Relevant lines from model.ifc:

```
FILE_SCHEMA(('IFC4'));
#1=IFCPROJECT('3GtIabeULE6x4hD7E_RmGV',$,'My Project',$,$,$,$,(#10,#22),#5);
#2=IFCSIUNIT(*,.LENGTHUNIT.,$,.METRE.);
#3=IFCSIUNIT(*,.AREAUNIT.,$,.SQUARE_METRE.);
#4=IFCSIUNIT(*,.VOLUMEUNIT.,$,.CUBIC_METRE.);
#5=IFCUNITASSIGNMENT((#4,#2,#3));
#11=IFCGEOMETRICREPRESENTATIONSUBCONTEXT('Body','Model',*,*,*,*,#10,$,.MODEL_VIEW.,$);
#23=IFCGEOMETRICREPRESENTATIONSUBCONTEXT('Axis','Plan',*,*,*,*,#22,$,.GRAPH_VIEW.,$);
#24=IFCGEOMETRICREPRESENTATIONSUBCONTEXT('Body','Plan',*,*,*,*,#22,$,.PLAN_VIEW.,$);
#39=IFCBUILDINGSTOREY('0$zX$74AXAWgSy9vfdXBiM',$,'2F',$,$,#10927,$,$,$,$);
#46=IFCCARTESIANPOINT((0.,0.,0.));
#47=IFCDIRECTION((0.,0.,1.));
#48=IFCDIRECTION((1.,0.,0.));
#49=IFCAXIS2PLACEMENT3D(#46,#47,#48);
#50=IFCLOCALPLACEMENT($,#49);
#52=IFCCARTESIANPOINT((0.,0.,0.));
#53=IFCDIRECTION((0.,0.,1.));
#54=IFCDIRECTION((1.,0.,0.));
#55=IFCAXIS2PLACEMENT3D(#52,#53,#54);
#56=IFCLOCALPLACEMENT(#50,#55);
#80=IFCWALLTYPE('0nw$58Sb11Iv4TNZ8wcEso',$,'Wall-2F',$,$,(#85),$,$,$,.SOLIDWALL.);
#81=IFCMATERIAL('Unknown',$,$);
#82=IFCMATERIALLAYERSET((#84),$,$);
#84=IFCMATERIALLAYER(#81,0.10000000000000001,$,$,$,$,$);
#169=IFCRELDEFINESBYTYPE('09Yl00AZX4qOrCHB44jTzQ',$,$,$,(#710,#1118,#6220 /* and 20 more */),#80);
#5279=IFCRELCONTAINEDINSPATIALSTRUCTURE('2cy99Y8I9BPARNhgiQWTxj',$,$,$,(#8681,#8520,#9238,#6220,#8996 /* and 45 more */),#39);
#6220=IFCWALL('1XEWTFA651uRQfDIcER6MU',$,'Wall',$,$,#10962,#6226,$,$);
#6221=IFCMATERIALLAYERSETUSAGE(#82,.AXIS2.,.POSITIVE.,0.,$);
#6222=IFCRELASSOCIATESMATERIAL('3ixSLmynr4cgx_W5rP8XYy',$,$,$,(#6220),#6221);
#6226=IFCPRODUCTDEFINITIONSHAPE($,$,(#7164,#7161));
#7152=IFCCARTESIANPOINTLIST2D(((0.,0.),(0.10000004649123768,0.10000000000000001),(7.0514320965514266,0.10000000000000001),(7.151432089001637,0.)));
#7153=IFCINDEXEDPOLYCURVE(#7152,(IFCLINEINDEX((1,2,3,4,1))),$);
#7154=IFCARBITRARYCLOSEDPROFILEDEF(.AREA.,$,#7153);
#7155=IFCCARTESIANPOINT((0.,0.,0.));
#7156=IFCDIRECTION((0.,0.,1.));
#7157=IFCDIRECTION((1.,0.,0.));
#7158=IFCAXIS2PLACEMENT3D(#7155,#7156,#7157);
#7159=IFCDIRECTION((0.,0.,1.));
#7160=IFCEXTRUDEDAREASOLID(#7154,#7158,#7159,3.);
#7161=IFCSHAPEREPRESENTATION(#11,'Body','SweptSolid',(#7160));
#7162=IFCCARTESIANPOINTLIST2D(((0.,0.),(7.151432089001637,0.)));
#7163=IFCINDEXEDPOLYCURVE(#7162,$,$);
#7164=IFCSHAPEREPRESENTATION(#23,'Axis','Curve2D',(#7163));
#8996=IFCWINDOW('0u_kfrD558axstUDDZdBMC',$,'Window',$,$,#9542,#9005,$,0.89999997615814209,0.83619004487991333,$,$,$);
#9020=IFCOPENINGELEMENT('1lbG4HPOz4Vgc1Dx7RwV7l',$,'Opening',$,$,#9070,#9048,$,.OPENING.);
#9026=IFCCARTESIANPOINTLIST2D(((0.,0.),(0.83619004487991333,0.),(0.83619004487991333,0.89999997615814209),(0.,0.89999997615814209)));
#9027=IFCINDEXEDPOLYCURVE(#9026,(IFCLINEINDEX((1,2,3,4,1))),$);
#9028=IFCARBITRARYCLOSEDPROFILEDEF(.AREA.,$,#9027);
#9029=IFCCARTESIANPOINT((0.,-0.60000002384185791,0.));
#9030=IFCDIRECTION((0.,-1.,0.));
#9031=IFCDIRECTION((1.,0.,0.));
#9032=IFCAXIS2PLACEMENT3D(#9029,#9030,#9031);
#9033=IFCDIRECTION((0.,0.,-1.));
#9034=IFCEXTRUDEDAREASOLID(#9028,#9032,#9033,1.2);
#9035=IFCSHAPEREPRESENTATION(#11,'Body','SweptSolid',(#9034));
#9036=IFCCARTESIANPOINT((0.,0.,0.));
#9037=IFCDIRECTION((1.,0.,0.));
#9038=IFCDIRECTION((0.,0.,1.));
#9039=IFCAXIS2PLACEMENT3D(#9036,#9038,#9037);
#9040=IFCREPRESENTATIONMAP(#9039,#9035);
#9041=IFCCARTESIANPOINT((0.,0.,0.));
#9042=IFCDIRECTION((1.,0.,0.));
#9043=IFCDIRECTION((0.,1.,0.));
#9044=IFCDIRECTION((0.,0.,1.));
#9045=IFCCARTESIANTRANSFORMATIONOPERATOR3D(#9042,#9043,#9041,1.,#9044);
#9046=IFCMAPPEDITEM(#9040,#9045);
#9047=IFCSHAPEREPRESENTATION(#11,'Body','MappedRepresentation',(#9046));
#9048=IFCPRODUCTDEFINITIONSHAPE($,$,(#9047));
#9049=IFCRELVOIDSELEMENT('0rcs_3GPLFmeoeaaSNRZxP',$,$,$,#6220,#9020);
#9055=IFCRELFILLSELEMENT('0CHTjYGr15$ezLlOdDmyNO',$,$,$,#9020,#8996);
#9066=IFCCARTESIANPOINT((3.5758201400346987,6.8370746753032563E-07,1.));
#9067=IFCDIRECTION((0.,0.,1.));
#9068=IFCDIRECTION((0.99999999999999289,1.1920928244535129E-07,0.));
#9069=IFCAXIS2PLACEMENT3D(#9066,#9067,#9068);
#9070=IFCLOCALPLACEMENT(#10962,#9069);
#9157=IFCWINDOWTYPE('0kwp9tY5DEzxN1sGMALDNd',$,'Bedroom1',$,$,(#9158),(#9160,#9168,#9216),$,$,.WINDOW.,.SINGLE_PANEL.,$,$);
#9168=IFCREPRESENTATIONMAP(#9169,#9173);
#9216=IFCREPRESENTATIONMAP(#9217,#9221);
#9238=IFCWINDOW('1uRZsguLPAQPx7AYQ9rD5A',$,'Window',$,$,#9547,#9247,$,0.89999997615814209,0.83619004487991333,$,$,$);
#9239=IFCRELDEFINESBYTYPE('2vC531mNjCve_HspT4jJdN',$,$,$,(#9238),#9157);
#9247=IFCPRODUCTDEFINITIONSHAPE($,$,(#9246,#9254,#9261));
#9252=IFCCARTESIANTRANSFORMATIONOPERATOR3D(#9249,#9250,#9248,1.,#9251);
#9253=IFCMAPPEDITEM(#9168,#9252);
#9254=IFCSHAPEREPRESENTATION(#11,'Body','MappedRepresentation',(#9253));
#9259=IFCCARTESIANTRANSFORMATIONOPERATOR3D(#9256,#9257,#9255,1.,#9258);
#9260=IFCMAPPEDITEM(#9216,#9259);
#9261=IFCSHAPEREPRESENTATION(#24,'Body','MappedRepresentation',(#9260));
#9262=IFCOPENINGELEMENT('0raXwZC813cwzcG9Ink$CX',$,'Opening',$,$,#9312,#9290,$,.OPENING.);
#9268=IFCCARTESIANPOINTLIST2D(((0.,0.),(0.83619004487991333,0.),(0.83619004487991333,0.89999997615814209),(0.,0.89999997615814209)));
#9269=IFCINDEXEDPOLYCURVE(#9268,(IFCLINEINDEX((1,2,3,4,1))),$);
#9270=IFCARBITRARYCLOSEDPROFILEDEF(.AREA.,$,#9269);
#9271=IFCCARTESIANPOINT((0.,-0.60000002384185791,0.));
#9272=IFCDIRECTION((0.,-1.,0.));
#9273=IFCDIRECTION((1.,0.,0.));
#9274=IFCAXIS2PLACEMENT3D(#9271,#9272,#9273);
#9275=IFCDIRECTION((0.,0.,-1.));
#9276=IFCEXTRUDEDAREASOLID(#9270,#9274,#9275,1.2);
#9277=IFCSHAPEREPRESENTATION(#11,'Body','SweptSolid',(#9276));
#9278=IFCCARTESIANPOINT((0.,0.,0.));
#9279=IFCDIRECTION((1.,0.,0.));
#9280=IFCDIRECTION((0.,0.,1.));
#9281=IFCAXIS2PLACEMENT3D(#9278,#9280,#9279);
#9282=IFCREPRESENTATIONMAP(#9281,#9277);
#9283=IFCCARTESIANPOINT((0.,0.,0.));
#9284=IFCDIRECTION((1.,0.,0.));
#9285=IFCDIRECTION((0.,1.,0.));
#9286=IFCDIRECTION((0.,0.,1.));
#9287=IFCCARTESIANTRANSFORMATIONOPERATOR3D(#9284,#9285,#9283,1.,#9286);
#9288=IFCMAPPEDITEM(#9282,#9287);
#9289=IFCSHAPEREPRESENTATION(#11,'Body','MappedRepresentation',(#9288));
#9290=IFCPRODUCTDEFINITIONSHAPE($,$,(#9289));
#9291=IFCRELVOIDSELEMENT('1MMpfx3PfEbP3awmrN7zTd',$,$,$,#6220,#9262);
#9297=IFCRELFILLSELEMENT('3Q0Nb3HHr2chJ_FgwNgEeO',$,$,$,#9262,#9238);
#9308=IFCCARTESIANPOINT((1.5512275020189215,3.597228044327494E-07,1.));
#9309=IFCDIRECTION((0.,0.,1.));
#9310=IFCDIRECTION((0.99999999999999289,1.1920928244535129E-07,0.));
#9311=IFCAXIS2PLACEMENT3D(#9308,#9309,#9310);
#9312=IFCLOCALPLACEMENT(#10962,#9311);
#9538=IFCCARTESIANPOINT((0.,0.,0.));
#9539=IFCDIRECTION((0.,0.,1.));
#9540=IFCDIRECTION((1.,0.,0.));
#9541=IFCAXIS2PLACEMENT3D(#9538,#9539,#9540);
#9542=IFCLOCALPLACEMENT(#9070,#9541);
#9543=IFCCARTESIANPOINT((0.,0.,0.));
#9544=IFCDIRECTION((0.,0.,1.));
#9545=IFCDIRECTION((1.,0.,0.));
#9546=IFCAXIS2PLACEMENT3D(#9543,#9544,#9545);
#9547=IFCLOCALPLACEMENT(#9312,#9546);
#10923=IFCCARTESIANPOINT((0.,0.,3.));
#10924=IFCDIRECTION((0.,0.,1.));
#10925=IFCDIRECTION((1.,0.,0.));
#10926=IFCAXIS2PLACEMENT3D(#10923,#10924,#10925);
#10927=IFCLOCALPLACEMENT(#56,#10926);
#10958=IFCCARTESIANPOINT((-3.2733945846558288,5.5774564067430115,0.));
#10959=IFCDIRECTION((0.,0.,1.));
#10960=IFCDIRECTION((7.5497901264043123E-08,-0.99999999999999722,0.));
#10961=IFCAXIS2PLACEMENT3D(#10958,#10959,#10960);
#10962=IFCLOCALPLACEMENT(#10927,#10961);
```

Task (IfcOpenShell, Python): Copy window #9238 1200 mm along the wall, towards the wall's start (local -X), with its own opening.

```python
import ifcopenshell
import ifcopenshell.api.feature
import ifcopenshell.api.geometry
import ifcopenshell.api.root
import ifcopenshell.geom
import ifcopenshell.util.element
import ifcopenshell.util.placement
import ifcopenshell.util.shape

model = ifcopenshell.open("model.ifc")
settings = ifcopenshell.geom.settings()


def volume(element):
    """Net volume in cubic metres, openings subtracted."""
    shape = ifcopenshell.geom.create_shape(settings, element)
    return ifcopenshell.util.shape.get_volume(shape.geometry)


window = model.by_id(9238)
opening = window.FillsVoids[0].RelatingOpeningElement
wall = opening.VoidsElements[0].RelatingBuildingElement
before = volume(wall)
shift = ifcopenshell.util.placement.get_local_placement(wall.ObjectPlacement)[:3, 0] * -1.2

# copy_class copies the void relationship, type, container and properties, but no geometry.
new_opening = ifcopenshell.api.root.copy_class(model, product=opening)
new_opening.Representation = ifcopenshell.util.element.copy_deep(
    model, opening.Representation, exclude=["IfcGeometricRepresentationContext", "IfcRepresentationMap"]
)
new_window = ifcopenshell.api.root.copy_class(model, product=window)
new_window.Representation = ifcopenshell.util.element.copy_deep(
    model, window.Representation, exclude=["IfcGeometricRepresentationContext", "IfcRepresentationMap"]
)
ifcopenshell.api.feature.add_filling(model, opening=new_opening, element=new_window)

for old, new in ((opening, new_opening), (window, new_window)):
    matrix = ifcopenshell.util.placement.get_local_placement(old.ObjectPlacement)
    matrix[:3, 3] += shift
    ifcopenshell.api.geometry.edit_object_placement(model, product=new, matrix=matrix, is_si=False)

after = volume(wall)

print(f"wall volume {before:.3f} -> {after:.3f} m3")

model.write("model_v2.ifc")
```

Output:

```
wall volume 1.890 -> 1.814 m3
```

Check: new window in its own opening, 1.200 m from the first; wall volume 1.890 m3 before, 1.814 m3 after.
